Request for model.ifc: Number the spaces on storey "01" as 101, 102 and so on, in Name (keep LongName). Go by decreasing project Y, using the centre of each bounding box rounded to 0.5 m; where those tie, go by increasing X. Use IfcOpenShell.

First a look at what the model holds.

```python
import ifcopenshell
import ifcopenshell.util.element
import ifcopenshell.util.placement

model = ifcopenshell.open("model.ifc")
print(model.schema)
storey = next(s for s in model.by_type("IfcBuildingStorey") if s.Name == "01")
spaces = [e for e in ifcopenshell.util.element.get_decomposition(storey) if e.is_a("IfcSpace")]
for e in sorted(spaces, key=lambda e: e.id()):
    origin = ifcopenshell.util.placement.get_local_placement(e.ObjectPlacement)[:3, 3]
    print(e.id(), e.Name, e.LongName, origin.round(2) + 0.0, sep=" | ")
```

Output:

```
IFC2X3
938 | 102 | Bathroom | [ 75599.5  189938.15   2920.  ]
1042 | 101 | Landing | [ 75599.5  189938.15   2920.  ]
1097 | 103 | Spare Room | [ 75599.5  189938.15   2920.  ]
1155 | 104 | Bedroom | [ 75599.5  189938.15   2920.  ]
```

```python
import ifcopenshell
import ifcopenshell.geom
import ifcopenshell.util.element
import ifcopenshell.util.shape

model = ifcopenshell.open("model.ifc")
settings = ifcopenshell.geom.settings()
settings.set("use-world-coords", True)


def centre(element):
    shape = ifcopenshell.geom.create_shape(settings, element)
    return ifcopenshell.util.shape.get_bbox_centroid(shape.geometry)


storey = next(s for s in model.by_type("IfcBuildingStorey") if s.Name == "01")
spaces = [e for e in ifcopenshell.util.element.get_decomposition(storey) if e.is_a("IfcSpace")]

# Insertion points can sit at a corner or the storey origin, so sort by the geometry (in metres).
centres = {e: centre(e) for e in spaces}
spaces.sort(key=lambda e: (-round(centres[e][1] / 0.5), centres[e][0]))

for i, e in enumerate(spaces, start=1):
    number = f"1{i:02d}"
    e.Name = number
    print(e.id(), number)

model.write("model_rev.ifc")
```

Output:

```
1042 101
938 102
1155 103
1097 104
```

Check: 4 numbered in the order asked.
